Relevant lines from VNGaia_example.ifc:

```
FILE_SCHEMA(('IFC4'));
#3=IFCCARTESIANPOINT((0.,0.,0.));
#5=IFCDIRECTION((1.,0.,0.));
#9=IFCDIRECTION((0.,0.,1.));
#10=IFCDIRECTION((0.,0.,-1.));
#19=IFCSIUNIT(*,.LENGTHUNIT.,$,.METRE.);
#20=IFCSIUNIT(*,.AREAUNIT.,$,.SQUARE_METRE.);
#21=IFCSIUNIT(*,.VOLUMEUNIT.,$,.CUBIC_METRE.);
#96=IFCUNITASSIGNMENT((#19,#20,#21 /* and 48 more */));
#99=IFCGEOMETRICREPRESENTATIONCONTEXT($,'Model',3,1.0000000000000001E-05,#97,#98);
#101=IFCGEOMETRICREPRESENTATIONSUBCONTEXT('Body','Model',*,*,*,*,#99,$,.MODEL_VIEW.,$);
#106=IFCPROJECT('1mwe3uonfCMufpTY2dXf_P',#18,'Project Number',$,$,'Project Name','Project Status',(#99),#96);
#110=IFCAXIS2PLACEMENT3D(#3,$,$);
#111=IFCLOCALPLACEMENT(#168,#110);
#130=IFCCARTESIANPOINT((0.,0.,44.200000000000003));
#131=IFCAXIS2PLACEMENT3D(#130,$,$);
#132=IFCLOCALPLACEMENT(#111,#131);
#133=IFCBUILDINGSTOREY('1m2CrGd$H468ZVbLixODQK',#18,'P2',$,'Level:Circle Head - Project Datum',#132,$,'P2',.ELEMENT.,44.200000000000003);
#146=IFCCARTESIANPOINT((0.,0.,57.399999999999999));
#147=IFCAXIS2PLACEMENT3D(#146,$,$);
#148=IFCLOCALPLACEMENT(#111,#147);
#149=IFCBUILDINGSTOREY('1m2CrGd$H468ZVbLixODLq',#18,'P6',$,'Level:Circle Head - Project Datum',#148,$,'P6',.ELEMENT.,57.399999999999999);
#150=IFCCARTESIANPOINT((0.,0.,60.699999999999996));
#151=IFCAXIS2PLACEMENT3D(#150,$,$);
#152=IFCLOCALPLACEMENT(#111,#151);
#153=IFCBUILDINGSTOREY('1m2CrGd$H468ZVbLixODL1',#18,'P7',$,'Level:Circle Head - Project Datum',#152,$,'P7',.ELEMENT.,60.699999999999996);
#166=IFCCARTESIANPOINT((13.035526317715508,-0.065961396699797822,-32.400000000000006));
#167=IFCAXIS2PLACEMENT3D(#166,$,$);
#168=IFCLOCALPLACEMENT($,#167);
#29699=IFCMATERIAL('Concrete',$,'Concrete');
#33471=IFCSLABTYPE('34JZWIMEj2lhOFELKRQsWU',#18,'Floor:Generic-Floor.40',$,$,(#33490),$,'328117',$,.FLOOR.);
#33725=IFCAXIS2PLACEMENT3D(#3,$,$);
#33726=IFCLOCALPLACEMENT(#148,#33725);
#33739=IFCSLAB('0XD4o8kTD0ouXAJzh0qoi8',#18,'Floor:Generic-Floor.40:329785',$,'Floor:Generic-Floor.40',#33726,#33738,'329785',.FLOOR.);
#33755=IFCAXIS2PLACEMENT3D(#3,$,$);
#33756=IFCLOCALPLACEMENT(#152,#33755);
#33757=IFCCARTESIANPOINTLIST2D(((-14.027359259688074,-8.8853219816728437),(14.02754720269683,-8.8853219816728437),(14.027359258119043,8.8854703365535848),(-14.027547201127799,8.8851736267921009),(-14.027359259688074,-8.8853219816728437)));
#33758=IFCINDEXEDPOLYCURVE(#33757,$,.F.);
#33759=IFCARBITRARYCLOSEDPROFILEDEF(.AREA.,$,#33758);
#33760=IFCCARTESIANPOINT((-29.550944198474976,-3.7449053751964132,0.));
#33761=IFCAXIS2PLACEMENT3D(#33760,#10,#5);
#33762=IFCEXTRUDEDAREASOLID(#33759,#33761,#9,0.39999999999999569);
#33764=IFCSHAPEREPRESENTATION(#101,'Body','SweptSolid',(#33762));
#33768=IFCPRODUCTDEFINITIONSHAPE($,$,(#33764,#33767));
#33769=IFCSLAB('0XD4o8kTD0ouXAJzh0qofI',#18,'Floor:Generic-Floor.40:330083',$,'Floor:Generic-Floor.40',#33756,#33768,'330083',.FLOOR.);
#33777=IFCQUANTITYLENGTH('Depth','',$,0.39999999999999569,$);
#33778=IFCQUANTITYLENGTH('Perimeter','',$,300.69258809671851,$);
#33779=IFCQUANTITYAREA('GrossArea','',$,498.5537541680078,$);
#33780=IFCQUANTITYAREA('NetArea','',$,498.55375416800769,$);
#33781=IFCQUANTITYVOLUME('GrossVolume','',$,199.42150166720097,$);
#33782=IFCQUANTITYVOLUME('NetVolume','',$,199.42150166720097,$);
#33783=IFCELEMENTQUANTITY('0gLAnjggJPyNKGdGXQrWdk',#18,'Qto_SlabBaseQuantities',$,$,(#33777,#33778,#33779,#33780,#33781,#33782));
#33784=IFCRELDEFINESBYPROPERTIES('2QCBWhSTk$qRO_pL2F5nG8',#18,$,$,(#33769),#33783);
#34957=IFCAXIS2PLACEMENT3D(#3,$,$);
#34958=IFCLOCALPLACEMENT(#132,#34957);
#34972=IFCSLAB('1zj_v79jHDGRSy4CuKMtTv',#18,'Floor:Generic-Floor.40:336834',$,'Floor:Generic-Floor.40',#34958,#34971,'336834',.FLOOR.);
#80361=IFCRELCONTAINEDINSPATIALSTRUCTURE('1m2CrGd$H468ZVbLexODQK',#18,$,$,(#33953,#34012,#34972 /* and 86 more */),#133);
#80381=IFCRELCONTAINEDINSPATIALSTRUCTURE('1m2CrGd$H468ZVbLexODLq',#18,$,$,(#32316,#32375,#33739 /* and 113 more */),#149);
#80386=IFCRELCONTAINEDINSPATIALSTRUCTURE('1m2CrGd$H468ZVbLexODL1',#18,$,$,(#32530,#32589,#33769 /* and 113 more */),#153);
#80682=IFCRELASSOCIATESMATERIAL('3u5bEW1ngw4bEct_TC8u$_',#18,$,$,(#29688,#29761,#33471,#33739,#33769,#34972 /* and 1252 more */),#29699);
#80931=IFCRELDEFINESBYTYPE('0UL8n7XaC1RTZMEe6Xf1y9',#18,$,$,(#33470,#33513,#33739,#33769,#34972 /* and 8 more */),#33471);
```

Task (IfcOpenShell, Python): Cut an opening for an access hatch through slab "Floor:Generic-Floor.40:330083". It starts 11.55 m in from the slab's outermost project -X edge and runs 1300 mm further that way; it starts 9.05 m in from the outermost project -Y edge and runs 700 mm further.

```python
import numpy as np
import ifcopenshell
import ifcopenshell.api.feature
import ifcopenshell.api.geometry
import ifcopenshell.api.pset
import ifcopenshell.api.root
import ifcopenshell.geom
import ifcopenshell.util.element
import ifcopenshell.util.placement
import ifcopenshell.util.representation
import ifcopenshell.util.shape
import ifcopenshell.util.unit

model = ifcopenshell.open("VNGaia_example.ifc")
unit_scale = ifcopenshell.util.unit.calculate_unit_scale(model)
area_scale = ifcopenshell.util.unit.calculate_unit_scale(model, "AREAUNIT")
volume_scale = ifcopenshell.util.unit.calculate_unit_scale(model, "VOLUMEUNIT")
settings = ifcopenshell.geom.settings()


def volume(element):
    """Net volume in cubic metres, openings subtracted."""
    shape = ifcopenshell.geom.create_shape(settings, element)
    return ifcopenshell.util.shape.get_volume(shape.geometry)


slab = model.by_guid("0XD4o8kTD0ouXAJzh0qofI")
before = volume(slab)

# Extent in the slab's own axes, in metres. The edges named are its -X and -Y sides.
slab_shape = ifcopenshell.geom.create_shape(settings, slab)
vertices = ifcopenshell.util.shape.get_vertices(slab_shape.geometry)
x_min, y_min, bottom = vertices.min(axis=0)
top = vertices[:, 2].max()

opening = ifcopenshell.api.root.create_entity(model, ifc_class="IfcOpeningElement", name="Access hatch opening", predefined_type="OPENING")
context = ifcopenshell.util.representation.get_context(model, "Model", "Body", "MODEL_VIEW")
width, depth = 1.3, 0.7
outline = [(0.0, 0.0), (width, 0.0), (width, depth), (0.0, depth), (0.0, 0.0)]
# Overshoot both faces by 50 mm so the cut is clean.
shape = ifcopenshell.api.geometry.add_slab_representation(
    model, context=context, depth=top - bottom + 0.1, polyline=outline
)
ifcopenshell.api.geometry.assign_representation(model, product=opening, representation=shape)

matrix = ifcopenshell.util.placement.get_local_placement(slab.ObjectPlacement)
matrix[:, 3] = matrix @ np.append(np.array([x_min + 11.55, y_min + 9.05, bottom - 0.05]) / unit_scale, 1.0)
ifcopenshell.api.geometry.edit_object_placement(model, product=opening, matrix=matrix, is_si=False)
ifcopenshell.api.feature.add_feature(model, feature=opening, element=slab)

after = volume(slab)

# Update the slab's stored quantities.
qto = model.by_id(ifcopenshell.util.element.get_pset(slab, "Qto_SlabBaseQuantities", should_inherit=False)["id"])
ifcopenshell.api.pset.edit_qto(model, qto=qto, properties={
    "NetArea": after / (top - bottom) / area_scale,
    "NetVolume": after / volume_scale,
})

print(f"slab volume {before:.3f} -> {after:.3f} m3")

model.write("VNGaia_example-out.ifc")
```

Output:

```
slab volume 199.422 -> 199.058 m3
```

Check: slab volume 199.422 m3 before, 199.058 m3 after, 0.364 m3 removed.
